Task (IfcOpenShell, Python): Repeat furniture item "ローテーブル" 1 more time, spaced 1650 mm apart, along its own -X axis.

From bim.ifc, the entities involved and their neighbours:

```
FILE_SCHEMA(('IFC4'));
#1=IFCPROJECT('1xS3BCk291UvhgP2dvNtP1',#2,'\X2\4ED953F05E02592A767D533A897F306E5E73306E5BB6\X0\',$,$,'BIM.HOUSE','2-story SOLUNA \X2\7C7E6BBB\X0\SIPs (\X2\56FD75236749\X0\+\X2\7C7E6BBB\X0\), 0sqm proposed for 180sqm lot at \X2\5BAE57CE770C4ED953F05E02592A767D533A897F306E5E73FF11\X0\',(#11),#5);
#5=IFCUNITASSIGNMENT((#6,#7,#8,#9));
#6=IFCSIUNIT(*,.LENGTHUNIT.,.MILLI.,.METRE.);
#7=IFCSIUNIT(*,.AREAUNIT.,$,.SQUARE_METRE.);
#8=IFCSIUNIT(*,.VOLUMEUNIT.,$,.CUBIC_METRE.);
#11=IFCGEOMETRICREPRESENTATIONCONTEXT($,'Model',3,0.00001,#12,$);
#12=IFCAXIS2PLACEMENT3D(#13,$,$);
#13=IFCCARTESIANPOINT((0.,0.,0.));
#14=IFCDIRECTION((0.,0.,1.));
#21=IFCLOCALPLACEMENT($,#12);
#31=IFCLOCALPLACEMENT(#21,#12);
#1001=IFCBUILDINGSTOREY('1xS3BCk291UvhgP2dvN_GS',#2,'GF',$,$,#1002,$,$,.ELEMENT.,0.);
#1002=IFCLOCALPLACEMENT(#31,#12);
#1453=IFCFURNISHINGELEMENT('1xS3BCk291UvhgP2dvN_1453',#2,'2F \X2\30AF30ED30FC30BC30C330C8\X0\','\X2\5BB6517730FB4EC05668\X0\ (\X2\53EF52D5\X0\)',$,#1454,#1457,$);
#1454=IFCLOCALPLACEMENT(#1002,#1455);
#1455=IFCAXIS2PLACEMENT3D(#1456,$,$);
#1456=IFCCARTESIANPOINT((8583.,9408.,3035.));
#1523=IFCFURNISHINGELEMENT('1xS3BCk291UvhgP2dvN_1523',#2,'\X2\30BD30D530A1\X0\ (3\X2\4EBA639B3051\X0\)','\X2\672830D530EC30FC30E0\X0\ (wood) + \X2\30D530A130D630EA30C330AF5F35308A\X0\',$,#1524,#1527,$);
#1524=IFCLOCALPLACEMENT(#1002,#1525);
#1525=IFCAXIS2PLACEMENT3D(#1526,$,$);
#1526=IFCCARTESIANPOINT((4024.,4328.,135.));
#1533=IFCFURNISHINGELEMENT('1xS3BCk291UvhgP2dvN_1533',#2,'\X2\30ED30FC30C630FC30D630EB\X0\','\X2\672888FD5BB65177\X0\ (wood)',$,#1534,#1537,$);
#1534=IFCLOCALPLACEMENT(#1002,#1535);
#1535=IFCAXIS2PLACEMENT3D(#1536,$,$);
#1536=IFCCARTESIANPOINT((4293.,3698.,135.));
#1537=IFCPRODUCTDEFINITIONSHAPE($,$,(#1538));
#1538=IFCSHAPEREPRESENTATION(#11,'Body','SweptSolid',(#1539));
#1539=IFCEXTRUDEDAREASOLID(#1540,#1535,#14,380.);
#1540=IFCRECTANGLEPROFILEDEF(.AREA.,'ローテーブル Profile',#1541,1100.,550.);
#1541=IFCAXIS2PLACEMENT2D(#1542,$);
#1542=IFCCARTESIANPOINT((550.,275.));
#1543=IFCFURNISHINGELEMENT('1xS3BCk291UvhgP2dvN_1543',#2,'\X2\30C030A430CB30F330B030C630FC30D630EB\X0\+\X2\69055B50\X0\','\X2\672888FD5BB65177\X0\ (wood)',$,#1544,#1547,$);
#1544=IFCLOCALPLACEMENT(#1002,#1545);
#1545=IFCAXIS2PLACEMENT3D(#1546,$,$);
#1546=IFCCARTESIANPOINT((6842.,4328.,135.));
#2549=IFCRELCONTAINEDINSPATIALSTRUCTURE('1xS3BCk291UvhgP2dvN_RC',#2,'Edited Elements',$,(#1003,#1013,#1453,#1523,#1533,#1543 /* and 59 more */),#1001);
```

```python
import ifcopenshell
import ifcopenshell.api.geometry
import ifcopenshell.api.root
import ifcopenshell.util.element
import ifcopenshell.util.placement

model = ifcopenshell.open("bim.ifc")


def reuse_history(source, copy):
    """copy_class also copies each property set's owner history, people and application; keep the originals."""
    for rel in copy.IsDefinedBy:
        if rel.is_a("IfcRelDefinesByProperties") and (history := rel.RelatingPropertyDefinition.OwnerHistory):
            rel.RelatingPropertyDefinition.OwnerHistory = source.OwnerHistory
            ifcopenshell.util.element.remove_deep2(model, history)


source = model.by_id(1533)
base = ifcopenshell.util.placement.get_local_placement(source.ObjectPlacement)
step = -base[:3, 0] * 1650.0

for i in range(1, 2):
    copy = ifcopenshell.api.root.copy_class(model, product=source)
    copy.Representation = ifcopenshell.util.element.copy_deep(
        model, source.Representation, exclude=["IfcGeometricRepresentationContext", "IfcRepresentationMap"]
    )
    reuse_history(source, copy)
    matrix = base.copy()
    matrix[:3, 3] += i * step
    print("added at", matrix[:3, 3].round(3) + 0.0)
    ifcopenshell.api.geometry.edit_object_placement(model, product=copy, matrix=matrix, is_si=False)

model.write("bim_rev.ifc")
```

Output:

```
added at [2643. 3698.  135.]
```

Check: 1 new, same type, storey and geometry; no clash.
